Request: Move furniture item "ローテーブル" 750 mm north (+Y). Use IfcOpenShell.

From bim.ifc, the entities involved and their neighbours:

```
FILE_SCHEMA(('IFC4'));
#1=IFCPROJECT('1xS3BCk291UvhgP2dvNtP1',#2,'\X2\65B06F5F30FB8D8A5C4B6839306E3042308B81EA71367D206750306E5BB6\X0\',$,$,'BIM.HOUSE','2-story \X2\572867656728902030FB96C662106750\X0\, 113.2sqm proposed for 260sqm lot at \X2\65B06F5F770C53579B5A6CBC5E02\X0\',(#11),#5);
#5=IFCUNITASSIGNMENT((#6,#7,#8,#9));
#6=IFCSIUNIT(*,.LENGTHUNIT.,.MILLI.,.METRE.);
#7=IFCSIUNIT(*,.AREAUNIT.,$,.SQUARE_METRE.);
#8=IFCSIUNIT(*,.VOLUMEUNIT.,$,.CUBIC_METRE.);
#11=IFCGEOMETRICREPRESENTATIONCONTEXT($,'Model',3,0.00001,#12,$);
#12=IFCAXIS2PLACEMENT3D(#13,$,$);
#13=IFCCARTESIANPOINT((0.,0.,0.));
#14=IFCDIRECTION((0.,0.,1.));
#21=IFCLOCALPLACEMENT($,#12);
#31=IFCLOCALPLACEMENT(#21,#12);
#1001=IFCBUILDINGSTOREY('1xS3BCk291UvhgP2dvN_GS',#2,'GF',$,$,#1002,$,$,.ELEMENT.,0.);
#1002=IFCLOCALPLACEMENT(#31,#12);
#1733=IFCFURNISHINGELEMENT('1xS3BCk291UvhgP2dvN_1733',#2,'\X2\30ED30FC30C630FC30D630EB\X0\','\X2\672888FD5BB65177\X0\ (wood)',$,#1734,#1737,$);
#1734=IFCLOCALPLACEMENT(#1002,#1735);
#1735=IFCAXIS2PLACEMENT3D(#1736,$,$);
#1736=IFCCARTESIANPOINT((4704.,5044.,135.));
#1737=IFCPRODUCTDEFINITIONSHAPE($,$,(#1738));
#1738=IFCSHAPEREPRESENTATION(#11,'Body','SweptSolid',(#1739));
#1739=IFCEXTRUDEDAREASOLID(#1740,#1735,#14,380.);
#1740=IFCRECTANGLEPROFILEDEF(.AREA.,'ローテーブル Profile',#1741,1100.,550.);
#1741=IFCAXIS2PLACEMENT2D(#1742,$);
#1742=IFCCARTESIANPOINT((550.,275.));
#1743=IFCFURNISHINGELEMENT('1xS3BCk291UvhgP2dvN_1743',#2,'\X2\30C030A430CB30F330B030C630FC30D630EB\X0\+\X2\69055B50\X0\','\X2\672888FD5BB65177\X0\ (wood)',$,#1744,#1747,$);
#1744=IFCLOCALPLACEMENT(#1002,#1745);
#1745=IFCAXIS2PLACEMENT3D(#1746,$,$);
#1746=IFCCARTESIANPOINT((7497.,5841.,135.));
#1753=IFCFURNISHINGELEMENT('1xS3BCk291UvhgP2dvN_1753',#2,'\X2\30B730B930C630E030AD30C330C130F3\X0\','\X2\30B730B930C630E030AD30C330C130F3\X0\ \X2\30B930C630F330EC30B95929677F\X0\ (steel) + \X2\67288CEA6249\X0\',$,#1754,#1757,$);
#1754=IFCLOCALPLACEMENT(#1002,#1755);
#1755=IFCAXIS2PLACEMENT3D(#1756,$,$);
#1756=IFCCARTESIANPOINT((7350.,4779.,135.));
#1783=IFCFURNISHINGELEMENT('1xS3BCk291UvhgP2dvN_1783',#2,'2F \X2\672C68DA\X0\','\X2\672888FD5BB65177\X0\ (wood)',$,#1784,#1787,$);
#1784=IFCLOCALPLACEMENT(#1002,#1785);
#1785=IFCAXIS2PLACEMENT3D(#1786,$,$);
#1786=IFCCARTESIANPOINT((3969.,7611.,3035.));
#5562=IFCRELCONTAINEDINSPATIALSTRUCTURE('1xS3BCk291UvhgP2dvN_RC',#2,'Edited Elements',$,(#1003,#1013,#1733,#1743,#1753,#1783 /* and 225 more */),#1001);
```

```python
import ifcopenshell
import ifcopenshell.api.geometry
import ifcopenshell.util.placement

model = ifcopenshell.open("bim.ifc")

item = model.by_id(1733)
matrix = ifcopenshell.util.placement.get_local_placement(item.ObjectPlacement)
matrix[1, 3] += 750.0
ifcopenshell.api.geometry.edit_object_placement(model, product=item, matrix=matrix, is_si=False)

print(ifcopenshell.util.placement.get_local_placement(item.ObjectPlacement).round(3) + 0.0)

model.write("bim_edited.ifc")
```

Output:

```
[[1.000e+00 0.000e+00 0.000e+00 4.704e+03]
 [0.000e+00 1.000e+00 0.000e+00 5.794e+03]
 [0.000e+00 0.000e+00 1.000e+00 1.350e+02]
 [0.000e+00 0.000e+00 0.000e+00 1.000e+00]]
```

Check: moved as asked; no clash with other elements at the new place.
